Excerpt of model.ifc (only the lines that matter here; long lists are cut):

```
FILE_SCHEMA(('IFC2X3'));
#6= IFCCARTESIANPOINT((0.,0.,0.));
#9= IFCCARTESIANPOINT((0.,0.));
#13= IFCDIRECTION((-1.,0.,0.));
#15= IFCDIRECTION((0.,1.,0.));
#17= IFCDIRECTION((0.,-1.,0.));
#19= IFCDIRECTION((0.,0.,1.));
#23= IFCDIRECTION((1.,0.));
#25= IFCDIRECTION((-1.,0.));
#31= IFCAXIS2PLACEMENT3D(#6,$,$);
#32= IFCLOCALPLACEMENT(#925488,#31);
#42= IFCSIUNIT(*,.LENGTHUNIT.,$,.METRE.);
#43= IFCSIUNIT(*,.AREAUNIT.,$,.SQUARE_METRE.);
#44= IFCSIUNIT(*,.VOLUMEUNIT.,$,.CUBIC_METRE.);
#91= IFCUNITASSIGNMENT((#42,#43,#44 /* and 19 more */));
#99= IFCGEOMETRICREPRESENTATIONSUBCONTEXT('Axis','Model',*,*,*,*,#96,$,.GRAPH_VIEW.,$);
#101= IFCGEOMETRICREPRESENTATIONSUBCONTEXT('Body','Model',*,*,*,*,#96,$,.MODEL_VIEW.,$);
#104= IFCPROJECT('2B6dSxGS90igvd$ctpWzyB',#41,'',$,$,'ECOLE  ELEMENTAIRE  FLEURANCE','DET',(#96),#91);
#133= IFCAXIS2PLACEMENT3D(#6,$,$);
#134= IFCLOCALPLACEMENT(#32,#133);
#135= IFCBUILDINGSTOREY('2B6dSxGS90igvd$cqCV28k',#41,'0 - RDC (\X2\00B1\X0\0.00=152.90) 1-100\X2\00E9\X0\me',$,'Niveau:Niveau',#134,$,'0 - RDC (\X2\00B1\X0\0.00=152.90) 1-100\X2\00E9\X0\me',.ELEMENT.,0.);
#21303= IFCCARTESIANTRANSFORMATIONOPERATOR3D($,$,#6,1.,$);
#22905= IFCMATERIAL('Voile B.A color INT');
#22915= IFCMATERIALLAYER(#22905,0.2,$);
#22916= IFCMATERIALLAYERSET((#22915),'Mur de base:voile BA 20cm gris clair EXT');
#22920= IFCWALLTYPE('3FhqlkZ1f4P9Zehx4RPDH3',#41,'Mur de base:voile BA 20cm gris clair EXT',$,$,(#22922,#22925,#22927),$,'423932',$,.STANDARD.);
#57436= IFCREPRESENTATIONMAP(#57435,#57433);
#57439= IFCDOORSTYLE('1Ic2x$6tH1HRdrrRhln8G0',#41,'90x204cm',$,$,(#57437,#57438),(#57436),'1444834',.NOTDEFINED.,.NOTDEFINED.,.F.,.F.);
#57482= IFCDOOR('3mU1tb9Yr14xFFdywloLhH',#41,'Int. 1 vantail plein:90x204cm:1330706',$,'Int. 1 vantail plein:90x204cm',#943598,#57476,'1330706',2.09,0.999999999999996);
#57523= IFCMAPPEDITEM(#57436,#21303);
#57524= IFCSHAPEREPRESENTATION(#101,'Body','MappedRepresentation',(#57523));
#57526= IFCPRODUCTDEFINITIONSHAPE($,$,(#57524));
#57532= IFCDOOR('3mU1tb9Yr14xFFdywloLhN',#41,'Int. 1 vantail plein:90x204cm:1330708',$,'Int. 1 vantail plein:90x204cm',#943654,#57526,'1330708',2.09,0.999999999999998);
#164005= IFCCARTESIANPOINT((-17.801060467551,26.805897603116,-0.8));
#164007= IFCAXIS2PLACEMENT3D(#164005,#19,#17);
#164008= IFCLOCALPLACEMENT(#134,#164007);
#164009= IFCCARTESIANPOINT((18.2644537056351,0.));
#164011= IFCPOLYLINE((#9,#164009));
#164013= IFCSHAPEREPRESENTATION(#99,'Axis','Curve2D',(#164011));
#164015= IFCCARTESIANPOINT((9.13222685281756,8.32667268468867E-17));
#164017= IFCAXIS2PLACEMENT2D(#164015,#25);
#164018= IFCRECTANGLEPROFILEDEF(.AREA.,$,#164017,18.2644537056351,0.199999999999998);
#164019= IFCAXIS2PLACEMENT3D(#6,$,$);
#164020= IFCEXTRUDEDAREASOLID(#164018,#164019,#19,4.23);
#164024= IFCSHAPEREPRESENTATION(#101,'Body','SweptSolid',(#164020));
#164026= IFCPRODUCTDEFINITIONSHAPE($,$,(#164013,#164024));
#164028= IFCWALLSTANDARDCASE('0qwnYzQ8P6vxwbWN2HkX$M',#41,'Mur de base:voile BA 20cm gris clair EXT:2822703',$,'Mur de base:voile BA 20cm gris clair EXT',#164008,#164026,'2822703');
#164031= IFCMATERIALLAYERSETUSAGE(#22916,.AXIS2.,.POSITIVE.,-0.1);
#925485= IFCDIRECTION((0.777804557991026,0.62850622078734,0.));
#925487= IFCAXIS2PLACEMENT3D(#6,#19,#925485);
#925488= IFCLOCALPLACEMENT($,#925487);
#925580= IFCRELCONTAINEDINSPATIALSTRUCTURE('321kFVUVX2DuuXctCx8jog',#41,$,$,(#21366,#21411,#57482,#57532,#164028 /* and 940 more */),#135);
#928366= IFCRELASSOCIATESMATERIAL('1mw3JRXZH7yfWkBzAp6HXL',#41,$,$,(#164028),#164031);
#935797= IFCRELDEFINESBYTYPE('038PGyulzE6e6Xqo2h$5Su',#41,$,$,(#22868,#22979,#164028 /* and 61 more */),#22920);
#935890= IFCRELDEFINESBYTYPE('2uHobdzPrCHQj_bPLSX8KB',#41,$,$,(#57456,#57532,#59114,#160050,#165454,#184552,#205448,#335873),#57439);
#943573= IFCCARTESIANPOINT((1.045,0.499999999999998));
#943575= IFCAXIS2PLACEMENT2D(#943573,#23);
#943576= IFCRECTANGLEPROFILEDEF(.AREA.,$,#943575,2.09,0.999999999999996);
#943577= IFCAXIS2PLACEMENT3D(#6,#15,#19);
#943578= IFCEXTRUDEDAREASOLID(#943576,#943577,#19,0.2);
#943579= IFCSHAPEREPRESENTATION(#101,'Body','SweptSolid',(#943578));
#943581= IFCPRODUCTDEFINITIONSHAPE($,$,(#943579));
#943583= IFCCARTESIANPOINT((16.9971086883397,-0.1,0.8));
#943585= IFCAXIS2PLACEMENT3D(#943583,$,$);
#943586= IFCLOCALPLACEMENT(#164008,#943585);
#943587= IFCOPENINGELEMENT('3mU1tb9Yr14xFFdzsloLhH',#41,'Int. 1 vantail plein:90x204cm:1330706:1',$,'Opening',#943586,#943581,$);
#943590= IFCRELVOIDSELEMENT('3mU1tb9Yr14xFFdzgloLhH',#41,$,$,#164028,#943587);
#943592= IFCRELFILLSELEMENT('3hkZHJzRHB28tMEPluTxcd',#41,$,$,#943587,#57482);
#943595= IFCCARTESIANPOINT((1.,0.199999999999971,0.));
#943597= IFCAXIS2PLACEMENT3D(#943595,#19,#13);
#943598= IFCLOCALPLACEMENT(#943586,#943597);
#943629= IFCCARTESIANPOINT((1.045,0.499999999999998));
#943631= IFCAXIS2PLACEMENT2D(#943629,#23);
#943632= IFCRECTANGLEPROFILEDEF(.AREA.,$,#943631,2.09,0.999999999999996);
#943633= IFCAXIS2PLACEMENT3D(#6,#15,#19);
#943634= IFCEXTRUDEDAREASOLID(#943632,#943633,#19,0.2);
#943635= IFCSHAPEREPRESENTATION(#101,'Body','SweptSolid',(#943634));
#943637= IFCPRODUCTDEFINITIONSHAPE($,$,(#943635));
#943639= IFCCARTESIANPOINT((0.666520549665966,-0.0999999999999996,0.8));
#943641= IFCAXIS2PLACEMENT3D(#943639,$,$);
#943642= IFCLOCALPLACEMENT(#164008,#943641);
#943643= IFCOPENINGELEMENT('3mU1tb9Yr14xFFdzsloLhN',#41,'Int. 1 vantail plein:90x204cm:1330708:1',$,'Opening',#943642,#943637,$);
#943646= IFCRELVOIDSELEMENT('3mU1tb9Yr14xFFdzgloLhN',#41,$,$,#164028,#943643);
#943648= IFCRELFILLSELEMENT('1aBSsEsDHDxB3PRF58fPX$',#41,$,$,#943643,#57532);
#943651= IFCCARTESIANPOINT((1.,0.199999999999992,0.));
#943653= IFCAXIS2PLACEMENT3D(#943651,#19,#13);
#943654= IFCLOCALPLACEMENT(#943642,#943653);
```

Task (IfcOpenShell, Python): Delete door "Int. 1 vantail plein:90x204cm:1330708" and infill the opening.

```python
import ifcopenshell
import ifcopenshell.api.feature
import ifcopenshell.api.root
import ifcopenshell.geom
import ifcopenshell.util.shape

model = ifcopenshell.open("model.ifc")
settings = ifcopenshell.geom.settings()


def volume(element):
    """Net volume in cubic metres, openings subtracted."""
    shape = ifcopenshell.geom.create_shape(settings, element)
    return ifcopenshell.util.shape.get_volume(shape.geometry)


door = model.by_guid("3mU1tb9Yr14xFFdywloLhN")
opening = door.FillsVoids[0].RelatingOpeningElement
wall = opening.VoidsElements[0].RelatingBuildingElement
before = volume(wall)

ifcopenshell.api.root.remove_product(model, product=door)
ifcopenshell.api.feature.remove_feature(model, feature=opening)

after = volume(wall)

print(f"wall volume {before:.3f} -> {after:.3f} m3")

model.write("model_v2.ifc")
```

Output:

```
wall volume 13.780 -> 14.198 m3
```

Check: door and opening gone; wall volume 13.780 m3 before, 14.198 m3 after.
